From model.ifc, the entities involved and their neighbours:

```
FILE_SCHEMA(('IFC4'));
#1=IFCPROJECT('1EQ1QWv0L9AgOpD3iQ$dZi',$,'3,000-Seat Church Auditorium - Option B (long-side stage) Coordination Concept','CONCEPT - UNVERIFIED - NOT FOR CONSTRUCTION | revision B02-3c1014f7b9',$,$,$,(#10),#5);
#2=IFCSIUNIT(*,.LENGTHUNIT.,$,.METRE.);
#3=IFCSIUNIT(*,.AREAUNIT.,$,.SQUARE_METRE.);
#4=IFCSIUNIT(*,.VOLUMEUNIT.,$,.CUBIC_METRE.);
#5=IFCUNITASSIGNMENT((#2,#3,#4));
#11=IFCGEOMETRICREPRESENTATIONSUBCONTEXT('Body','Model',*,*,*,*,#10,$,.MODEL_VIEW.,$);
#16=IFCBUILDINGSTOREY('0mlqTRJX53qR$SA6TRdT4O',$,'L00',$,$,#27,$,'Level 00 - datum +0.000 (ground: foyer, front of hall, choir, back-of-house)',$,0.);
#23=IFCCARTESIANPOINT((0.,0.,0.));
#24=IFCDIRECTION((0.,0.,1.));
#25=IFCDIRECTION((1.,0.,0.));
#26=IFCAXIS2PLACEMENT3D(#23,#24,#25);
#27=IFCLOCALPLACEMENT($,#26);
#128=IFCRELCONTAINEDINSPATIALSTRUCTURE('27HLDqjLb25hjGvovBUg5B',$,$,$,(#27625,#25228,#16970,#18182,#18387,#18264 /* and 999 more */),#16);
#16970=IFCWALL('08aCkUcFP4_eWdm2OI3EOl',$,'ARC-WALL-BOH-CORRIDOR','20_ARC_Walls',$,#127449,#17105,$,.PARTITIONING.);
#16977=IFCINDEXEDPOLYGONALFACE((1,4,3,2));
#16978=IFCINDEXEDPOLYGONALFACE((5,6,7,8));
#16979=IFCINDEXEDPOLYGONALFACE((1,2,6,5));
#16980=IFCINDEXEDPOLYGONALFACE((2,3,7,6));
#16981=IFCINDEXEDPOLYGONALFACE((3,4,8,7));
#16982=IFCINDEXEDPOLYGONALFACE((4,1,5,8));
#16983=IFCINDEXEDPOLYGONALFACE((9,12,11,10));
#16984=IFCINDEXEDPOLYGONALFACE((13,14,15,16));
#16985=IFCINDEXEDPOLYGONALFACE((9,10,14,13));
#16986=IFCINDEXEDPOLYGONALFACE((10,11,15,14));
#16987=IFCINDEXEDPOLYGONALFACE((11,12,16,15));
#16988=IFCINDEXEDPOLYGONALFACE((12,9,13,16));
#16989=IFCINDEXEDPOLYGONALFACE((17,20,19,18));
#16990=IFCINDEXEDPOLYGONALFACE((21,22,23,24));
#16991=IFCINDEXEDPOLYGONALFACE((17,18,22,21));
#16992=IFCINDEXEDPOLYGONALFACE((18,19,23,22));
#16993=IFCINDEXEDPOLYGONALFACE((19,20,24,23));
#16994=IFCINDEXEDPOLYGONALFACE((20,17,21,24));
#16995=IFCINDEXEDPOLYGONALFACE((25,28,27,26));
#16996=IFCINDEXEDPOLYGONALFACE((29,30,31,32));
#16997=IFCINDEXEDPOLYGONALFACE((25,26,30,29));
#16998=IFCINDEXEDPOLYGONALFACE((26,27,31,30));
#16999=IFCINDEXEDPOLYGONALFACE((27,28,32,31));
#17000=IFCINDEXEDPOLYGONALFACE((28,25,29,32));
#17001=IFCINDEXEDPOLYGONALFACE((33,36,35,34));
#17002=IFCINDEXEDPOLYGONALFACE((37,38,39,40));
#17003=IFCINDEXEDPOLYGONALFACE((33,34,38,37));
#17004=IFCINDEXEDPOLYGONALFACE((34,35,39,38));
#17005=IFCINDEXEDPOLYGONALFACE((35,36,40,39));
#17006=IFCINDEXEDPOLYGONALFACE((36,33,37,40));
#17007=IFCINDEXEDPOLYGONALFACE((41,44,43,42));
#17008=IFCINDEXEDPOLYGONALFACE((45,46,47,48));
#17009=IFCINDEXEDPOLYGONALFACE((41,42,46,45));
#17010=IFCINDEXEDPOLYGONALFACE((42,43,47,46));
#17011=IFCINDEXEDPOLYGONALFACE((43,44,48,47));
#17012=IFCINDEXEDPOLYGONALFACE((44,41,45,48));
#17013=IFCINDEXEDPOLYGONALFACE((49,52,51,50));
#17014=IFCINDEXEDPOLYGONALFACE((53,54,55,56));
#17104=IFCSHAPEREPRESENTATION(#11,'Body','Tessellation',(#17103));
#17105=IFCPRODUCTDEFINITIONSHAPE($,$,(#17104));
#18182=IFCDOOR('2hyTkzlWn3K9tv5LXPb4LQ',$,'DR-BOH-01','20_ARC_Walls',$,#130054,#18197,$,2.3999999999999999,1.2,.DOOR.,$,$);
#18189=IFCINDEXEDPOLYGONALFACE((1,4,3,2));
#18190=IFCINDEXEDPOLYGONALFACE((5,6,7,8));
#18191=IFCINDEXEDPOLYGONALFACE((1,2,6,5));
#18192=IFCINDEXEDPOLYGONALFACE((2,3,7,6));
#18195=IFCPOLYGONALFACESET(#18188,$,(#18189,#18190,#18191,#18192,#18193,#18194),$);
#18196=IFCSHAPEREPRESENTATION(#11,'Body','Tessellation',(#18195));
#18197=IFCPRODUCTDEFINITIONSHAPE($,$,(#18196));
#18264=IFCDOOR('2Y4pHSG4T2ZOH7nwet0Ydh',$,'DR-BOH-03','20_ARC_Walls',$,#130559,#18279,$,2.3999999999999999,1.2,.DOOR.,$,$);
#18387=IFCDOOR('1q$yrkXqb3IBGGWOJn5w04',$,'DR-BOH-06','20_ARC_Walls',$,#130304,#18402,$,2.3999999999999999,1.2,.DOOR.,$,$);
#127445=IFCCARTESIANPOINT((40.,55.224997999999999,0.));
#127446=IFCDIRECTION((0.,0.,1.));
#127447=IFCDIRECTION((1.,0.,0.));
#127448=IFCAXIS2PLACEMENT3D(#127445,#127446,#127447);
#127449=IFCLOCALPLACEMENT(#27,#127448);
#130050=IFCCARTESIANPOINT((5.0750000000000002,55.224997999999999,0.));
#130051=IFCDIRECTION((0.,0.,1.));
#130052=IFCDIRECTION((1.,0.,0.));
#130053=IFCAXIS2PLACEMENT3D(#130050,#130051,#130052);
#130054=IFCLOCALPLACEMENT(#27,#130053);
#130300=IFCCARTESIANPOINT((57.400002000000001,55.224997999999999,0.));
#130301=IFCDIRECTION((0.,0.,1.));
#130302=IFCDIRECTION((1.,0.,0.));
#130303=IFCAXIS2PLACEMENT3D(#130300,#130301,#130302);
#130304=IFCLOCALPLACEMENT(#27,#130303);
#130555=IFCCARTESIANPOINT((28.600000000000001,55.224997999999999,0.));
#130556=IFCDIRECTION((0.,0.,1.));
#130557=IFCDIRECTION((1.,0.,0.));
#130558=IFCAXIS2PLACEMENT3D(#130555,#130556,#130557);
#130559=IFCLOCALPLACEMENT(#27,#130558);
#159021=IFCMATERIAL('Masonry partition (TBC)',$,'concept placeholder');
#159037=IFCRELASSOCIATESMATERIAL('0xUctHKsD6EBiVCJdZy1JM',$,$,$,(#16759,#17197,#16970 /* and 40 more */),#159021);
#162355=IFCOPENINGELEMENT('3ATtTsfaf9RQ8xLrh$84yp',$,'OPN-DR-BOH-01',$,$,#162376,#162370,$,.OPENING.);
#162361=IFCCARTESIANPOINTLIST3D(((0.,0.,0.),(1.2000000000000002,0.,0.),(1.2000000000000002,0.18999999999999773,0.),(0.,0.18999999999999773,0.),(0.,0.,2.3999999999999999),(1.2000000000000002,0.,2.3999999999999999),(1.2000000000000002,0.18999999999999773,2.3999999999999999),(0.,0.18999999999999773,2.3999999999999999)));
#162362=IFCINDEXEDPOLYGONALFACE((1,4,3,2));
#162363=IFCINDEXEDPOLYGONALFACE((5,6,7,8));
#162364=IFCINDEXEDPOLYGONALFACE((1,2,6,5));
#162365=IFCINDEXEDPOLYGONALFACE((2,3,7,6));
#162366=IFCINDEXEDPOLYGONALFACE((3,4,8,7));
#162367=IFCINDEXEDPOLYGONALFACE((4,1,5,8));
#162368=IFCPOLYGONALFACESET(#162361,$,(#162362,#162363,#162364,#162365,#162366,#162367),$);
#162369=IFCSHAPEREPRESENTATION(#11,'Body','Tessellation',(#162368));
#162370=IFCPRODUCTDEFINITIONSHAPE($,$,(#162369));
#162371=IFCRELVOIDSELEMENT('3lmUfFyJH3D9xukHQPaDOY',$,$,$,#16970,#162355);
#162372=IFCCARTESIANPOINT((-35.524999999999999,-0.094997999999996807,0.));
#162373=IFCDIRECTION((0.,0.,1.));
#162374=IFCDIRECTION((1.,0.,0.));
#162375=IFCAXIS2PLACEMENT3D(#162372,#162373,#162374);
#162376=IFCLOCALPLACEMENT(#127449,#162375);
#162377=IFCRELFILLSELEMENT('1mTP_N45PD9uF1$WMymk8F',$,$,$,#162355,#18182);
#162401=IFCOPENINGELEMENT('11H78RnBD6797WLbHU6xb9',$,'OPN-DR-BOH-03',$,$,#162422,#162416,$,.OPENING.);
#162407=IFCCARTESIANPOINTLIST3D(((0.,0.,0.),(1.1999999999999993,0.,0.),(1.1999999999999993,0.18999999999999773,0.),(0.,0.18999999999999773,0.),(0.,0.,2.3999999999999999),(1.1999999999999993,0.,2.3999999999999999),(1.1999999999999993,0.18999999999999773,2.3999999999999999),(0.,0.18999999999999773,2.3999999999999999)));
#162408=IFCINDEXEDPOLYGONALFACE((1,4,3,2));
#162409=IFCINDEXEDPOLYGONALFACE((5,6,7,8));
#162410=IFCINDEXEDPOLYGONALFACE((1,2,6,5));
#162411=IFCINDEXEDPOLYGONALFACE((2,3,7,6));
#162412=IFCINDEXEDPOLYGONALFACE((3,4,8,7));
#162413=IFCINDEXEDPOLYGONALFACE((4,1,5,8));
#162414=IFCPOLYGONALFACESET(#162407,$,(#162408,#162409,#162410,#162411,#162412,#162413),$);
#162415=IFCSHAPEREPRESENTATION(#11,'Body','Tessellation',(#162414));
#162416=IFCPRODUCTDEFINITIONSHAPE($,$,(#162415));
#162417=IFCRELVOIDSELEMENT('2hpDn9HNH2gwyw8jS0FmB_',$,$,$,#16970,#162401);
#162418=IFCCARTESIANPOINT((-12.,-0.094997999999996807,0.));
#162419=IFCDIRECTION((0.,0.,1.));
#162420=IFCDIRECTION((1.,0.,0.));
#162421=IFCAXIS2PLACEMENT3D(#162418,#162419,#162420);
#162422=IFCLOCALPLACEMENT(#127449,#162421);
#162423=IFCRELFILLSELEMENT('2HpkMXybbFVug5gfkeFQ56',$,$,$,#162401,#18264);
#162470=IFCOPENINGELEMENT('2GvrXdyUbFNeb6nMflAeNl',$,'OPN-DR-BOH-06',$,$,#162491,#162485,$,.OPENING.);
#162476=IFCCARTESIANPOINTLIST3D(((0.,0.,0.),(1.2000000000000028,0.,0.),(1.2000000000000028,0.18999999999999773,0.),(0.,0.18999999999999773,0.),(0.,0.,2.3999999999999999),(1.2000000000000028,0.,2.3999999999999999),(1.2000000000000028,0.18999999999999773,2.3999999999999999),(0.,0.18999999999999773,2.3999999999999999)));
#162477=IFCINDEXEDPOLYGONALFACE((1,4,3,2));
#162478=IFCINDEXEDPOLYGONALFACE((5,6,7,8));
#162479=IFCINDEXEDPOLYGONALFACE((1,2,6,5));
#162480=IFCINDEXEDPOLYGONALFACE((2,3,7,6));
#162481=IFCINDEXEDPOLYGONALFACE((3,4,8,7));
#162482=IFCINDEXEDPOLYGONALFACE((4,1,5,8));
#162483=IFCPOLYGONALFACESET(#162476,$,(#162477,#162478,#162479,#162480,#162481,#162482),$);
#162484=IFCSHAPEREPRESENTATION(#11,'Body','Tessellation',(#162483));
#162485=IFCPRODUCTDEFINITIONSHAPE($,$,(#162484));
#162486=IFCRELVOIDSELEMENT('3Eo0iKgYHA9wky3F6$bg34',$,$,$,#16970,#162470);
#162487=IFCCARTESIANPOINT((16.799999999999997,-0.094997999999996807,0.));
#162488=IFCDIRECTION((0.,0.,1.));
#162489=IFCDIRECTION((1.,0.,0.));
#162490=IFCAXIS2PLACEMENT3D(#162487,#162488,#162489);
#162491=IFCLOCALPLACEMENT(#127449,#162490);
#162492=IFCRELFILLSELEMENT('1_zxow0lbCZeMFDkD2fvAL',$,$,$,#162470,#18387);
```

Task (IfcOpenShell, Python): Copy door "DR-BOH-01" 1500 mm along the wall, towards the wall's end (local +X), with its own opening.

```python
import ifcopenshell
import ifcopenshell.api.feature
import ifcopenshell.api.geometry
import ifcopenshell.api.root
import ifcopenshell.geom
import ifcopenshell.util.element
import ifcopenshell.util.placement
import ifcopenshell.util.shape
import ifcopenshell.util.unit

model = ifcopenshell.open("model.ifc")
unit_scale = ifcopenshell.util.unit.calculate_unit_scale(model)
settings = ifcopenshell.geom.settings()


def volume(element):
    """Net volume in cubic metres, openings subtracted."""
    shape = ifcopenshell.geom.create_shape(settings, element)
    return ifcopenshell.util.shape.get_volume(shape.geometry)


door = model.by_guid("2hyTkzlWn3K9tv5LXPb4LQ")
opening = door.FillsVoids[0].RelatingOpeningElement
wall = opening.VoidsElements[0].RelatingBuildingElement
before = volume(wall)
shift = ifcopenshell.util.placement.get_local_placement(wall.ObjectPlacement)[:3, 0] * 1.5 / unit_scale

# copy_class copies the void relationship, type, container and properties, but no geometry.
new_opening = ifcopenshell.api.root.copy_class(model, product=opening)
new_opening.Representation = ifcopenshell.util.element.copy_deep(
    model, opening.Representation, exclude=["IfcGeometricRepresentationContext", "IfcRepresentationMap"]
)
new_door = ifcopenshell.api.root.copy_class(model, product=door)
new_door.Representation = ifcopenshell.util.element.copy_deep(
    model, door.Representation, exclude=["IfcGeometricRepresentationContext", "IfcRepresentationMap"]
)
ifcopenshell.api.feature.add_filling(model, opening=new_opening, element=new_door)

for old, new in ((opening, new_opening), (door, new_door)):
    matrix = ifcopenshell.util.placement.get_local_placement(old.ObjectPlacement)
    matrix[:3, 3] += shift
    ifcopenshell.api.geometry.edit_object_placement(model, product=new, matrix=matrix, is_si=False)

after = volume(wall)

print(f"wall volume {before:.3f} -> {after:.3f} m3")

model.write("model_updated.ifc")
```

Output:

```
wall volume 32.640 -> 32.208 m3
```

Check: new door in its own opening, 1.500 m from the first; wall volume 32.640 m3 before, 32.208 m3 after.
